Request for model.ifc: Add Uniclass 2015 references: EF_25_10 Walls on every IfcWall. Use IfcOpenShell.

First a look at what the model holds.

```python
import ifcopenshell

model = ifcopenshell.open("model.ifc")
print(model.schema)
print("classifications:", [c.Name for c in model.by_type("IfcClassification")])
for ifc_class in ("IfcDoor", "IfcRoof", "IfcStair", "IfcWall", "IfcWindow"):
    print(ifc_class, len(model.by_type(ifc_class)))
```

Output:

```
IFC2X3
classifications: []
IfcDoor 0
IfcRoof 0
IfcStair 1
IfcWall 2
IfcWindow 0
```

```python
import ifcopenshell
import ifcopenshell.api.classification

model = ifcopenshell.open("model.ifc")

# IFC2X3 requires Source and Edition and has no link from the project to the system.
system = model.create_entity("IfcClassification", Source="NBS", Edition="2015", Name="Uniclass 2015")

codes = {
    "IfcWall": ("EF_25_10", "Walls"),
}
for ifc_class, (code, name) in codes.items():
    products = model.by_type(ifc_class)
    ifcopenshell.api.classification.add_reference(
        model, products=products, classification=system, identification=code, name=name
    )
    print(code, len(products))

model.write("model-out.ifc")
```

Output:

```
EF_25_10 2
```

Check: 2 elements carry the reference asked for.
